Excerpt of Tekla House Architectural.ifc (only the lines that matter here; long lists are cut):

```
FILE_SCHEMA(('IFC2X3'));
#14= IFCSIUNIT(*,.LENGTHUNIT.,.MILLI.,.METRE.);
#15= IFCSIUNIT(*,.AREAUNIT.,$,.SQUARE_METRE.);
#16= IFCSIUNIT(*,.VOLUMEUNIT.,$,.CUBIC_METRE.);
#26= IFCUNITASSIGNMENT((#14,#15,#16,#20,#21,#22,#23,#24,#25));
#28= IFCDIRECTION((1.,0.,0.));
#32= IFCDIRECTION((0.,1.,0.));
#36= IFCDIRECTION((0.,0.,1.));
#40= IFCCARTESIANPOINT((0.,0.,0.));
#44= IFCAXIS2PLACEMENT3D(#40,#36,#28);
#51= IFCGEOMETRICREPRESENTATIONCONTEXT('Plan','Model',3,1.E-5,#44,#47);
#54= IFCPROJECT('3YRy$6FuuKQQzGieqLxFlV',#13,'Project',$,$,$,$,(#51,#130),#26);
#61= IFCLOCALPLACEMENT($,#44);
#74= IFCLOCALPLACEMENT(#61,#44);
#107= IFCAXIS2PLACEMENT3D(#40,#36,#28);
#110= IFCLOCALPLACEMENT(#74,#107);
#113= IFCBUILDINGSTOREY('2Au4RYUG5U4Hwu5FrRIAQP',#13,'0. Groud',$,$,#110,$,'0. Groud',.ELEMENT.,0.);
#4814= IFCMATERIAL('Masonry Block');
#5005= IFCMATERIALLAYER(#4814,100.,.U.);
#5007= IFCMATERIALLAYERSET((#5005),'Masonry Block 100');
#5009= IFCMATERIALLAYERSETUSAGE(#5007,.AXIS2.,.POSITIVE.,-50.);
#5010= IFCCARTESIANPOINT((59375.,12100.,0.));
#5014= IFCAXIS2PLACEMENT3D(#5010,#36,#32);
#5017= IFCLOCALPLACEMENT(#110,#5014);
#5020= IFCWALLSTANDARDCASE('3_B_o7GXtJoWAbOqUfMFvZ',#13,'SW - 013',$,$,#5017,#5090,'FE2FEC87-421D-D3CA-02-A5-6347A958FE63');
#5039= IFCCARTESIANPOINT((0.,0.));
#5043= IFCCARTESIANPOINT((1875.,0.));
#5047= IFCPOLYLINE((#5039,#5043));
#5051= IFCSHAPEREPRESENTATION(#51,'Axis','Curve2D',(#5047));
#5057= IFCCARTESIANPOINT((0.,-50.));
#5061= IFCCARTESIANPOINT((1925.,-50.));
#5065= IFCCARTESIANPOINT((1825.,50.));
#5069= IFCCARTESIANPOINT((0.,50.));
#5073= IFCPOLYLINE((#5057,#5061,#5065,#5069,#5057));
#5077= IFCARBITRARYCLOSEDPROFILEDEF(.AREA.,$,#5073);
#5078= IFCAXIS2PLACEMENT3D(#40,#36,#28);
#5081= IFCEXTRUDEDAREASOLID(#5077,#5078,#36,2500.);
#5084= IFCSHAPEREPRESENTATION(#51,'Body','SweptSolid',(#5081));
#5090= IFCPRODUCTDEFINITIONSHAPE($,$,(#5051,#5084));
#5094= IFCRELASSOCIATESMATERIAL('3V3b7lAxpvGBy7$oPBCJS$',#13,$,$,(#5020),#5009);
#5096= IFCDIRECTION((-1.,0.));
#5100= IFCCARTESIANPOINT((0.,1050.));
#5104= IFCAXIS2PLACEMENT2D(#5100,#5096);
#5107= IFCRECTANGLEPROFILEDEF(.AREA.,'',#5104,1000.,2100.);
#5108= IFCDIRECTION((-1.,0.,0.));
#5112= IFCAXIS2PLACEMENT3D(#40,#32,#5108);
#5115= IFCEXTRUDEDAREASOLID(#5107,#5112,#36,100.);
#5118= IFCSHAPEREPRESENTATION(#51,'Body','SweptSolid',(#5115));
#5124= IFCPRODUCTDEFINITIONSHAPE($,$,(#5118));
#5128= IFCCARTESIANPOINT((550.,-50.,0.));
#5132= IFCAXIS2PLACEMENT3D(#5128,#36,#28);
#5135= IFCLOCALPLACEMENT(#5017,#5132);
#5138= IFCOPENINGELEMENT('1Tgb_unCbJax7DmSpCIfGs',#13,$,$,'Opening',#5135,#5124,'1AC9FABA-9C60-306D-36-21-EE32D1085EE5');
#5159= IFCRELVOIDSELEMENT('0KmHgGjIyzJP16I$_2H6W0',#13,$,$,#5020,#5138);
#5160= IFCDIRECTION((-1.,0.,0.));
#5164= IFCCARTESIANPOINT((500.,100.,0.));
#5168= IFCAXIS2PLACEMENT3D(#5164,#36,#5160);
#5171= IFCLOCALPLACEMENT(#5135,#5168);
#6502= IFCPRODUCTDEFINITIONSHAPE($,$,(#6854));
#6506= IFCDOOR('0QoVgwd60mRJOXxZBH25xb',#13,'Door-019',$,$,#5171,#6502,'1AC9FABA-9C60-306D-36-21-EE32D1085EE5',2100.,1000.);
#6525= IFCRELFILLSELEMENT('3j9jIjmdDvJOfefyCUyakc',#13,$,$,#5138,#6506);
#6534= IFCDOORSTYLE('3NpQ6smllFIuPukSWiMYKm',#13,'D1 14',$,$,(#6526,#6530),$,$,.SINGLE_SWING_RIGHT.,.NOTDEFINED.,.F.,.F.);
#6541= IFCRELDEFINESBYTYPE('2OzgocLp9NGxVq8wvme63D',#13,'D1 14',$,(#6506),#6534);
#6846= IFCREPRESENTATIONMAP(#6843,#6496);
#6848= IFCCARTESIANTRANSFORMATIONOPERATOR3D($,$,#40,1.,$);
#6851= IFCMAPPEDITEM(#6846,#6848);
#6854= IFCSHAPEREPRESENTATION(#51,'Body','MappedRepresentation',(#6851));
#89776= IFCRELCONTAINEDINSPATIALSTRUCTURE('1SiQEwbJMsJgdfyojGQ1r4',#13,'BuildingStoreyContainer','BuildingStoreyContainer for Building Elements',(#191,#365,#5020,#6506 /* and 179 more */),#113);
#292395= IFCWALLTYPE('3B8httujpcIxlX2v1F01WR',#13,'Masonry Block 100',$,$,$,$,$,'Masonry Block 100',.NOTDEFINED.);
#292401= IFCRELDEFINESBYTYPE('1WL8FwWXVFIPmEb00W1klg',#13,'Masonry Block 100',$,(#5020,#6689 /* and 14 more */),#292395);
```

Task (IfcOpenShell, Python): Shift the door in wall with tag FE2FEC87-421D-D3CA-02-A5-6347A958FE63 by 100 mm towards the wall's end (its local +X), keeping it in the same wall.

```python
import ifcopenshell
import ifcopenshell.api.geometry
import ifcopenshell.util.placement

model = ifcopenshell.open("Tekla House Architectural.ifc")

door = model.by_id(6506)
opening = door.FillsVoids[0].RelatingOpeningElement
wall = opening.VoidsElements[0].RelatingBuildingElement

wall_matrix = ifcopenshell.util.placement.get_local_placement(wall.ObjectPlacement)
shift = wall_matrix[:3, 0] * 100.0
before = ifcopenshell.util.placement.get_local_placement(door.ObjectPlacement)[:3, 3].copy()

# The door is placed relative to its opening, so it follows when the opening moves.
matrix = ifcopenshell.util.placement.get_local_placement(opening.ObjectPlacement)
matrix[:3, 3] += shift
ifcopenshell.api.geometry.edit_object_placement(
    model, product=opening, matrix=matrix, is_si=False, should_transform_children=True
)

after = ifcopenshell.util.placement.get_local_placement(door.ObjectPlacement)[:3, 3]
print("door moved by", (after - before).round(3) + 0.0)

model.write("Tekla House Architectural_edited.ifc")
```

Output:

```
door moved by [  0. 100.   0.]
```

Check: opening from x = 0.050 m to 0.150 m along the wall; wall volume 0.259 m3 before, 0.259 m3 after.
